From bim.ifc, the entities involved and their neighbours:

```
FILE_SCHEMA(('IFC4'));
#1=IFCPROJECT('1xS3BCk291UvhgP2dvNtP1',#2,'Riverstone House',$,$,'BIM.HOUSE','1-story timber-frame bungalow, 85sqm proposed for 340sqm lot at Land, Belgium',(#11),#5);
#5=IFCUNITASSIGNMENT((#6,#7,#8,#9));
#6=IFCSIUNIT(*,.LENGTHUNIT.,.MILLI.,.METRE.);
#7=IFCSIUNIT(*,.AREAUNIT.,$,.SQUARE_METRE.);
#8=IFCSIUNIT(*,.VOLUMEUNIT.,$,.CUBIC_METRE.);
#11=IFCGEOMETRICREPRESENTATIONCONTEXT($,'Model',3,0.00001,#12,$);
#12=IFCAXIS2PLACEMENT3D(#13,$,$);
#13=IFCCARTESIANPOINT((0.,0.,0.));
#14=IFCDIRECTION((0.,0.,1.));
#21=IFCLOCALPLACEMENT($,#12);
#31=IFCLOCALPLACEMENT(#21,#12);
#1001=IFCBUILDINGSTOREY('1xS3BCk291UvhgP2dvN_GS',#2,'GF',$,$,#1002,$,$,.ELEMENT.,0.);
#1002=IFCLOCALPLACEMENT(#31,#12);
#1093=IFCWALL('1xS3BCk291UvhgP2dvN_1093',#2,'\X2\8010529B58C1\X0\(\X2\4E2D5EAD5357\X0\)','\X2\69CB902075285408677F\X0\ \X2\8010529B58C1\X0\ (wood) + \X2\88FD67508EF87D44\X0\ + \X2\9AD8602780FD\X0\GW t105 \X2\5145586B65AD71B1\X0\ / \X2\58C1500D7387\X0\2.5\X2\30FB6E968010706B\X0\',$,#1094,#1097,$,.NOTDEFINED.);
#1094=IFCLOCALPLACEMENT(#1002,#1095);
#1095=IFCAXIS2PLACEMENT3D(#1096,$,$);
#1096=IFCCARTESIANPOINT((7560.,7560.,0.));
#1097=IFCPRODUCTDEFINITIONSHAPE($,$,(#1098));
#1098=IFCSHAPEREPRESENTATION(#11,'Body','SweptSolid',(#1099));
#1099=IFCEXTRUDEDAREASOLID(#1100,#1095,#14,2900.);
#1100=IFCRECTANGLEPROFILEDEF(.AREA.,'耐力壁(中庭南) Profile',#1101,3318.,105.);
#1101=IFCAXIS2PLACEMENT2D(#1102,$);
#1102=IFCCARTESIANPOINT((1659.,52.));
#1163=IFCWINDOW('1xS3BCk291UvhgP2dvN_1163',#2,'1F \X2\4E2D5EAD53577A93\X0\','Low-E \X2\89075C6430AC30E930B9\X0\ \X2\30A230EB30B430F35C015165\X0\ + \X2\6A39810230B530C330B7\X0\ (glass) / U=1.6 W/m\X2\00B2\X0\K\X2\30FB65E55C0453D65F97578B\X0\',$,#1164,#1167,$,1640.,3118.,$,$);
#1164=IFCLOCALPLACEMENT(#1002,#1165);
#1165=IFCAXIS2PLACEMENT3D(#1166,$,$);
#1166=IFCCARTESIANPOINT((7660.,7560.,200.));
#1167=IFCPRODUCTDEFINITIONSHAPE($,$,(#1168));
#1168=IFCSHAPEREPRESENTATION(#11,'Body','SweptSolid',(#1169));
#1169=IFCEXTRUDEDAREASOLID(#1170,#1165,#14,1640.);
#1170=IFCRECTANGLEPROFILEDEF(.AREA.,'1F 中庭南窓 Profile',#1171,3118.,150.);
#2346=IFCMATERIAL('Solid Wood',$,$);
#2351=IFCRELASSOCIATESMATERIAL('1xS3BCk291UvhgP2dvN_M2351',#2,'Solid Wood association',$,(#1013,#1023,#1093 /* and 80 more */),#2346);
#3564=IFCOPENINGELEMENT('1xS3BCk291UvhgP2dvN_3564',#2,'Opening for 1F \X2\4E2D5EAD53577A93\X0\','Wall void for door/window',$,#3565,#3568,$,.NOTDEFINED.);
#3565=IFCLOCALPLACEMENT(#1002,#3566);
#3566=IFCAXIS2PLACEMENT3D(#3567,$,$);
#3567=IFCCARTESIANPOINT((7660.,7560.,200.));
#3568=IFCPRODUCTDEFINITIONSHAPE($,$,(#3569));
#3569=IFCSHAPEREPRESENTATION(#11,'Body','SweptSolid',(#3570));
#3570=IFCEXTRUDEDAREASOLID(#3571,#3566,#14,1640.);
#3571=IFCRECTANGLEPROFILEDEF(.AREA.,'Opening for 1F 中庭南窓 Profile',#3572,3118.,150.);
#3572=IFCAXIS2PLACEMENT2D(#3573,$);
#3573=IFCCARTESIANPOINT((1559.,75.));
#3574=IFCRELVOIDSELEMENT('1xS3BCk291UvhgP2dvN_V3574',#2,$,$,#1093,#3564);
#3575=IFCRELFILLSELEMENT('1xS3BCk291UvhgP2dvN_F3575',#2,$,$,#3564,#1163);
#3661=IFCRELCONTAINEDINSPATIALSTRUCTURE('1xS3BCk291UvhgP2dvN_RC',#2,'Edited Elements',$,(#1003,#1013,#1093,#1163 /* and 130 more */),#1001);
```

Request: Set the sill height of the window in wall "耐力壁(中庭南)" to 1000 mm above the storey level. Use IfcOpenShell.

```python
import numpy as np
import ifcopenshell
import ifcopenshell.api.geometry
import ifcopenshell.geom
import ifcopenshell.util.element
import ifcopenshell.util.placement
import ifcopenshell.util.shape
import ifcopenshell.util.unit

model = ifcopenshell.open("bim.ifc")
unit_scale = ifcopenshell.util.unit.calculate_unit_scale(model)

window = model.by_guid("1xS3BCk291UvhgP2dvN_1163")
opening = window.FillsVoids[0].RelatingOpeningElement
storey = ifcopenshell.util.element.get_container(window, ifc_class="IfcBuildingStorey")
level = ifcopenshell.util.placement.get_local_placement(storey.ObjectPlacement)[2, 3]

# The opening's origin need not be at the sill, so measure its lowest point.
shape = ifcopenshell.geom.create_shape(ifcopenshell.geom.settings(), opening)
bottom = ifcopenshell.util.shape.get_shape_bottom_elevation(shape, shape.geometry) / unit_scale
dz = level + 1000.0 - bottom

shift = np.array([0.0, 0.0, dz])
# The window is not placed relative to its opening, so move both.
for product in (opening, window):
    matrix = ifcopenshell.util.placement.get_local_placement(product.ObjectPlacement)
    matrix[:3, 3] += shift
    ifcopenshell.api.geometry.edit_object_placement(model, product=product, matrix=matrix, is_si=False)

print(f"moved by {dz * unit_scale:+.3f} m")

model.write("bim_edited.ifc")
```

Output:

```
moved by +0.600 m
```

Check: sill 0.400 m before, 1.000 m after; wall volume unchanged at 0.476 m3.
